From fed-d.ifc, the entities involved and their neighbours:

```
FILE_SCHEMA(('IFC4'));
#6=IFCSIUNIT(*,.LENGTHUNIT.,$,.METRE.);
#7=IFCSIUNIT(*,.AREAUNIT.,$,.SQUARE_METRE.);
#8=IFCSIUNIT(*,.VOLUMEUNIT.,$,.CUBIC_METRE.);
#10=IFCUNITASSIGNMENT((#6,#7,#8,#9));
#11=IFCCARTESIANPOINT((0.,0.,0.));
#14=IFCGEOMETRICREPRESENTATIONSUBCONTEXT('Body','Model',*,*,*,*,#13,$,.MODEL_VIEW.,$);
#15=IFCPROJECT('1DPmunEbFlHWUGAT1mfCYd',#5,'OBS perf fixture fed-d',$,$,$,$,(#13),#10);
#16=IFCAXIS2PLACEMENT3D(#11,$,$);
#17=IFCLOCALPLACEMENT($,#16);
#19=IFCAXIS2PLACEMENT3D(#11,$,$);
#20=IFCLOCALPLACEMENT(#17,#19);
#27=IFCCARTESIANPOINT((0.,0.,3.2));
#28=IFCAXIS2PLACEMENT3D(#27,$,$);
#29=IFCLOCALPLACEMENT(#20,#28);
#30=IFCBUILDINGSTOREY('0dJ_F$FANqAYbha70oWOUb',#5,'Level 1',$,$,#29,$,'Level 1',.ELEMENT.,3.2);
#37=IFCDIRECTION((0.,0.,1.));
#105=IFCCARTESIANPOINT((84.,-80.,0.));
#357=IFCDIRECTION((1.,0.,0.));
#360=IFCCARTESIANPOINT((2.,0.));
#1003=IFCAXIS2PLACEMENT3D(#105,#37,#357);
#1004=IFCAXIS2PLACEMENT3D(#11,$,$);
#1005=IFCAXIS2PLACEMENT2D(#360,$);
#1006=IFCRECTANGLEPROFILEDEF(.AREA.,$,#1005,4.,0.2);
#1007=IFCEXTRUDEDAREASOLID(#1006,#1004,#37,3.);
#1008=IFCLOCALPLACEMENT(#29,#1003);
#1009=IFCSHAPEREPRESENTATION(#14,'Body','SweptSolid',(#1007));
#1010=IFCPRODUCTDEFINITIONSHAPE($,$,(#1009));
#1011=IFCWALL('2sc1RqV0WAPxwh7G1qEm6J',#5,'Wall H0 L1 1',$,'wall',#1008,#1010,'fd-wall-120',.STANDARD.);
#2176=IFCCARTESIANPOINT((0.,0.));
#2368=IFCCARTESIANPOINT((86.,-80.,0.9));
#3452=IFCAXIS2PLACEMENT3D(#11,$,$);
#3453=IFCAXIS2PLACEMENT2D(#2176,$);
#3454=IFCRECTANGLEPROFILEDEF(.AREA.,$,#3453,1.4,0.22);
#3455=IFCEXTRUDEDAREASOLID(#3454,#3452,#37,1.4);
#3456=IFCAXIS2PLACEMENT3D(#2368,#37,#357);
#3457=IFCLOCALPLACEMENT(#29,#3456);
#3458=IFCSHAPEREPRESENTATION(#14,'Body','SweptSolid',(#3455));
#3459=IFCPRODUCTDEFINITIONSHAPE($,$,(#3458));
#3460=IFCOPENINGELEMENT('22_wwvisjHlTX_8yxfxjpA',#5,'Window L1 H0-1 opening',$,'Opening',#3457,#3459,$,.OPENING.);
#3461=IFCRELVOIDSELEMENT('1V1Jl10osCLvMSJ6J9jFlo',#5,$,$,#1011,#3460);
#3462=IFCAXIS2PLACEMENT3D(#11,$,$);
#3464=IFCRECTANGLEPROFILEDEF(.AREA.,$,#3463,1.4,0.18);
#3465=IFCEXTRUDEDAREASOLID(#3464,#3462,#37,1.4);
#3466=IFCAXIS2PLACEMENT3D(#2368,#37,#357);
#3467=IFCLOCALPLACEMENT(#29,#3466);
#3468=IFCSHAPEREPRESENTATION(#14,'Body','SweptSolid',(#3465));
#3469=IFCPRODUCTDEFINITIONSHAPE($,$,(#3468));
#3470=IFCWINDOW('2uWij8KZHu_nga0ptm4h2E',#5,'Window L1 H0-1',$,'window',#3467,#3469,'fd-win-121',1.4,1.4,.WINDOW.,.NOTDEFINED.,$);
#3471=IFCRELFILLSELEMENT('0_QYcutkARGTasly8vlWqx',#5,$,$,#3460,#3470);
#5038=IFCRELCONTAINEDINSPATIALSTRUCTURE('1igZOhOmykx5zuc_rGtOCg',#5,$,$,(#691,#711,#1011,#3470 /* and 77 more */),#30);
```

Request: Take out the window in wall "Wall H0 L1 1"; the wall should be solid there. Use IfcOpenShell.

```python
import ifcopenshell
import ifcopenshell.api.feature
import ifcopenshell.api.root
import ifcopenshell.geom
import ifcopenshell.util.shape

model = ifcopenshell.open("fed-d.ifc")
settings = ifcopenshell.geom.settings()


def volume(element):
    """Net volume in cubic metres, openings subtracted."""
    shape = ifcopenshell.geom.create_shape(settings, element)
    return ifcopenshell.util.shape.get_volume(shape.geometry)


window = model.by_guid("2uWij8KZHu_nga0ptm4h2E")
opening = window.FillsVoids[0].RelatingOpeningElement
wall = opening.VoidsElements[0].RelatingBuildingElement
before = volume(wall)

ifcopenshell.api.root.remove_product(model, product=window)
ifcopenshell.api.feature.remove_feature(model, feature=opening)

after = volume(wall)

print(f"wall volume {before:.3f} -> {after:.3f} m3")

model.write("fed-d-out.ifc")
```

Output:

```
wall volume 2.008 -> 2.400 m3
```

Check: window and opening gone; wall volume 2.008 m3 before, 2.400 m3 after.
